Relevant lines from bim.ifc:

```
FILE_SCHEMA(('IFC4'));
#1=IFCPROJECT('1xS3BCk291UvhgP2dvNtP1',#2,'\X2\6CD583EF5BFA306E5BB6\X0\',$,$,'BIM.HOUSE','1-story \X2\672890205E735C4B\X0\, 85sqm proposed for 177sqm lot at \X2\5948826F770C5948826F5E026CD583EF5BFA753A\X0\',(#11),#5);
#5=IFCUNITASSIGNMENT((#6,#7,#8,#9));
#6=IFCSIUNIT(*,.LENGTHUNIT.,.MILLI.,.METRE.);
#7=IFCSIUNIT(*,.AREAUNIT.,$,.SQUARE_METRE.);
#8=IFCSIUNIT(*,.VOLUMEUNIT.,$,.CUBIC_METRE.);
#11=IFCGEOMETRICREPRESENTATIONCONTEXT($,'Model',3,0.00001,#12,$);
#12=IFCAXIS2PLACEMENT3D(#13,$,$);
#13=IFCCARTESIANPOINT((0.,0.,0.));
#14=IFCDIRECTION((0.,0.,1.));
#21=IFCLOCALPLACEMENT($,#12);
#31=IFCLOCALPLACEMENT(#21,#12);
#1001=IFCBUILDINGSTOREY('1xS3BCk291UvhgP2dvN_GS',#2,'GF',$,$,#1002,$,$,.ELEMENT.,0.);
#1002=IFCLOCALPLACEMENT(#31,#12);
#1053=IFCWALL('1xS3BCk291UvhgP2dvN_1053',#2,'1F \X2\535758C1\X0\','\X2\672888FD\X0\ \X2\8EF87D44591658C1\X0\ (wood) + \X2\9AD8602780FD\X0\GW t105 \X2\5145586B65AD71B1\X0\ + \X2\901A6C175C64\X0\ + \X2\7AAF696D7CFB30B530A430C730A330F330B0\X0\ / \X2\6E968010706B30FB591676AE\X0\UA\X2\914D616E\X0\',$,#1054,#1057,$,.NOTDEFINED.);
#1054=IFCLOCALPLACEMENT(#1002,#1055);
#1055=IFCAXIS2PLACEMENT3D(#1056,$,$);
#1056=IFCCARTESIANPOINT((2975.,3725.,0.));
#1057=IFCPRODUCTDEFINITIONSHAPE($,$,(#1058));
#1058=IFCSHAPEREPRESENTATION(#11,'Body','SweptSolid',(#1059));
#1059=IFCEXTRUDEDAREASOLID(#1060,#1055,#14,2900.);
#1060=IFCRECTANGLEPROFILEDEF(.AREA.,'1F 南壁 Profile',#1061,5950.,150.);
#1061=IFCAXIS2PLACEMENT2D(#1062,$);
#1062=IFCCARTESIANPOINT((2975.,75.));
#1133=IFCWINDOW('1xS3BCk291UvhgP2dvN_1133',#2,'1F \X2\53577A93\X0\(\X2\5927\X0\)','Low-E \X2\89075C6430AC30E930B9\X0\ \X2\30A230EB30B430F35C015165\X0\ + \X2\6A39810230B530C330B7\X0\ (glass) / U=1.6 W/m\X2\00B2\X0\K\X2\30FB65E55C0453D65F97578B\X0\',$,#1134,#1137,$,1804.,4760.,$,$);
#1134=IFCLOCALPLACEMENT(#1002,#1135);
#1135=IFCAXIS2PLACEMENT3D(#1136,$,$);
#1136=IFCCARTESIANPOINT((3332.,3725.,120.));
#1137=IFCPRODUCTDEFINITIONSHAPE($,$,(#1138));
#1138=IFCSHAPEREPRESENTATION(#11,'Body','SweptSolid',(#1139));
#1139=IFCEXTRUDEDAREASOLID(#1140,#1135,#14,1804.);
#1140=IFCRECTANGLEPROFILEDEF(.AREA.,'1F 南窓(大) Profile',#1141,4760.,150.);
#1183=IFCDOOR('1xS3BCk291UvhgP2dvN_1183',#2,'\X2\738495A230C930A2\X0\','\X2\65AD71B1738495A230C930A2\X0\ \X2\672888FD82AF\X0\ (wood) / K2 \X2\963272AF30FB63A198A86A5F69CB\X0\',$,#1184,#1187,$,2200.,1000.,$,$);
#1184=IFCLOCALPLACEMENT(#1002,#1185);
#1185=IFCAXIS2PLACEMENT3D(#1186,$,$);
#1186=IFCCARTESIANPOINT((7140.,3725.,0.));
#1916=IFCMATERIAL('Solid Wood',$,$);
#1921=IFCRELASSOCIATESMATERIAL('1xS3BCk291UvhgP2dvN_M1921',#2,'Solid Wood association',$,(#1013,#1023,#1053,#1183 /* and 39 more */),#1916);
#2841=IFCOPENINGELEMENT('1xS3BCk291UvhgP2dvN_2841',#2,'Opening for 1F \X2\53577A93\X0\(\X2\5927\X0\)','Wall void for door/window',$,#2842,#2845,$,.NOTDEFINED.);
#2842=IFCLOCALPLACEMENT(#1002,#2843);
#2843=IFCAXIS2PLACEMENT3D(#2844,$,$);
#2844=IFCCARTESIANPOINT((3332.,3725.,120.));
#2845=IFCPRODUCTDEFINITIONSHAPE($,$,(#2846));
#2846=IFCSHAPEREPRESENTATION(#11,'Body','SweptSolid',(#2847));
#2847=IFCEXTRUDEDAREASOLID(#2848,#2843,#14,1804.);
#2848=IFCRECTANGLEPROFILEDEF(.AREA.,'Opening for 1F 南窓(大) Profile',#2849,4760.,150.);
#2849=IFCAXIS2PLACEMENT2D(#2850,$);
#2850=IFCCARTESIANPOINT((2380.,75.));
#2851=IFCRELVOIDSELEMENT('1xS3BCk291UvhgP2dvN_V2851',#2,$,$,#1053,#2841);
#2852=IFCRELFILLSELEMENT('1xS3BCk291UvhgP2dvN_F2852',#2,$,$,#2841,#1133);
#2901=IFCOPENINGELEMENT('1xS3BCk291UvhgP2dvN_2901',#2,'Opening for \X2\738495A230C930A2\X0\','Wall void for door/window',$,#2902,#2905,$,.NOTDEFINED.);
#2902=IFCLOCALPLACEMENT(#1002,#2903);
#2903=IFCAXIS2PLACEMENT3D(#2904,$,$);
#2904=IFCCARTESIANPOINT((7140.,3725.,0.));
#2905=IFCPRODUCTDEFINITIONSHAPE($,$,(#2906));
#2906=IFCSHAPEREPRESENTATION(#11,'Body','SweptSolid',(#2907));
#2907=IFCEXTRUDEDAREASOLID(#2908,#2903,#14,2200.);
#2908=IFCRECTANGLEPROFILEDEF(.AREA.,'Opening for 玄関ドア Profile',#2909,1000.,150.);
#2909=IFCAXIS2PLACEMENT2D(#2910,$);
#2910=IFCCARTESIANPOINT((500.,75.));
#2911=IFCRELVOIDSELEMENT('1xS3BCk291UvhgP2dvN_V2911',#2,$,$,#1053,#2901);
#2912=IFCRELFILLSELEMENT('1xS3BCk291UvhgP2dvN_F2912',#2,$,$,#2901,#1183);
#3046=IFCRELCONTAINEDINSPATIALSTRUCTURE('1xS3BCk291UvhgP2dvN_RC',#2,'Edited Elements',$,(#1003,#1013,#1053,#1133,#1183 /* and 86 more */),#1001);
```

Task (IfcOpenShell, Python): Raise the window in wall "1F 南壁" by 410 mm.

```python
import numpy as np
import ifcopenshell
import ifcopenshell.api.geometry
import ifcopenshell.util.placement
import ifcopenshell.util.unit

model = ifcopenshell.open("bim.ifc")
unit_scale = ifcopenshell.util.unit.calculate_unit_scale(model)

window = model.by_guid("1xS3BCk291UvhgP2dvN_1133")
opening = window.FillsVoids[0].RelatingOpeningElement
dz = 0.41 / unit_scale

shift = np.array([0.0, 0.0, dz])
# The window is not placed relative to its opening, so move both.
for product in (opening, window):
    matrix = ifcopenshell.util.placement.get_local_placement(product.ObjectPlacement)
    matrix[:3, 3] += shift
    ifcopenshell.api.geometry.edit_object_placement(model, product=product, matrix=matrix, is_si=False)

print(f"moved by {dz * unit_scale:+.3f} m")

model.write("bim_edited.ifc")
```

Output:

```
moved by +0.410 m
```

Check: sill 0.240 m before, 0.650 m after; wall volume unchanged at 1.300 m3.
